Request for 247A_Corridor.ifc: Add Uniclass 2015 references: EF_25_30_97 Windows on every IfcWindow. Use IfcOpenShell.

First a look at what the model holds.

```python
import ifcopenshell

model = ifcopenshell.open("247A_Corridor.ifc")
print(model.schema)
print("classifications:", [c.Name for c in model.by_type("IfcClassification")])
for ifc_class in ("IfcDoor", "IfcRoof", "IfcStair", "IfcWall", "IfcWindow"):
    print(ifc_class, len(model.by_type(ifc_class)))
```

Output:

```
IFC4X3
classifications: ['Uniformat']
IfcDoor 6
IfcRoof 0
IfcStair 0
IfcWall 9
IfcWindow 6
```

```python
import ifcopenshell
import ifcopenshell.api.classification

model = ifcopenshell.open("247A_Corridor.ifc")

system = ifcopenshell.api.classification.add_classification(model, classification="Uniclass 2015")

codes = {
    "IfcWindow": ("EF_25_30_97", "Windows"),
}
for ifc_class, (code, name) in codes.items():
    products = model.by_type(ifc_class)
    ifcopenshell.api.classification.add_reference(
        model, products=products, classification=system, identification=code, name=name
    )
    print(code, len(products))

model.write("247A_Corridor_edited.ifc")
```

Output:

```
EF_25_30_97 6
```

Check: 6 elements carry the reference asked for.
